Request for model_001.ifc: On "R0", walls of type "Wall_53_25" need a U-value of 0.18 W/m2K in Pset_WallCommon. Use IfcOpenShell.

First a look at what the model holds.

```python
import ifcopenshell
import ifcopenshell.util.element

model = ifcopenshell.open("model_001.ifc")
print(model.schema)
storey = next(s for s in model.by_type("IfcBuildingStorey") if s.Name == "R0")
walls = [e for e in ifcopenshell.util.element.get_decomposition(storey) if e.is_a("IfcWall")]
seen = {}
for e in walls:
    element_type = ifcopenshell.util.element.get_type(e)
    key = (element_type.Name if element_type != e and element_type else None, ifcopenshell.util.element.get_pset(e, "Pset_WallCommon", "ThermalTransmittance"))
    seen[key] = seen.get(key, 0) + 1
for (name, value), count in sorted(seen.items(), key=str):
    print(count, "x", name, "|", value)
```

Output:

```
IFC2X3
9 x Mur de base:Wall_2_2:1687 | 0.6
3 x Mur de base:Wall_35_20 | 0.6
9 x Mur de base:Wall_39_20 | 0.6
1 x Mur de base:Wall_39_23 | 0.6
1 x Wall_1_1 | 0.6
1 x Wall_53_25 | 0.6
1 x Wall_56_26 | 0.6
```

```python
import ifcopenshell
import ifcopenshell.api.pset
import ifcopenshell.util.element

model = ifcopenshell.open("model_001.ifc")

storey = next(s for s in model.by_type("IfcBuildingStorey") if s.Name == "R0")
walls = [e for e in ifcopenshell.util.element.get_decomposition(storey) if e.is_a("IfcWall")]

count = 0
for e in walls:
    element_type = ifcopenshell.util.element.get_type(e)
    if element_type in (None, e) or element_type.Name != "Wall_53_25":
        continue
    # add_pset returns the element's existing set when there is one.
    pset = ifcopenshell.api.pset.add_pset(model, product=e, name="Pset_WallCommon")
    ifcopenshell.api.pset.edit_pset(model, pset=pset, properties={"ThermalTransmittance": 0.18})
    count += 1

print(count, "walls updated")

model.write("model_001-out.ifc")
```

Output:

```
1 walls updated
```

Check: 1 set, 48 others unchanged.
